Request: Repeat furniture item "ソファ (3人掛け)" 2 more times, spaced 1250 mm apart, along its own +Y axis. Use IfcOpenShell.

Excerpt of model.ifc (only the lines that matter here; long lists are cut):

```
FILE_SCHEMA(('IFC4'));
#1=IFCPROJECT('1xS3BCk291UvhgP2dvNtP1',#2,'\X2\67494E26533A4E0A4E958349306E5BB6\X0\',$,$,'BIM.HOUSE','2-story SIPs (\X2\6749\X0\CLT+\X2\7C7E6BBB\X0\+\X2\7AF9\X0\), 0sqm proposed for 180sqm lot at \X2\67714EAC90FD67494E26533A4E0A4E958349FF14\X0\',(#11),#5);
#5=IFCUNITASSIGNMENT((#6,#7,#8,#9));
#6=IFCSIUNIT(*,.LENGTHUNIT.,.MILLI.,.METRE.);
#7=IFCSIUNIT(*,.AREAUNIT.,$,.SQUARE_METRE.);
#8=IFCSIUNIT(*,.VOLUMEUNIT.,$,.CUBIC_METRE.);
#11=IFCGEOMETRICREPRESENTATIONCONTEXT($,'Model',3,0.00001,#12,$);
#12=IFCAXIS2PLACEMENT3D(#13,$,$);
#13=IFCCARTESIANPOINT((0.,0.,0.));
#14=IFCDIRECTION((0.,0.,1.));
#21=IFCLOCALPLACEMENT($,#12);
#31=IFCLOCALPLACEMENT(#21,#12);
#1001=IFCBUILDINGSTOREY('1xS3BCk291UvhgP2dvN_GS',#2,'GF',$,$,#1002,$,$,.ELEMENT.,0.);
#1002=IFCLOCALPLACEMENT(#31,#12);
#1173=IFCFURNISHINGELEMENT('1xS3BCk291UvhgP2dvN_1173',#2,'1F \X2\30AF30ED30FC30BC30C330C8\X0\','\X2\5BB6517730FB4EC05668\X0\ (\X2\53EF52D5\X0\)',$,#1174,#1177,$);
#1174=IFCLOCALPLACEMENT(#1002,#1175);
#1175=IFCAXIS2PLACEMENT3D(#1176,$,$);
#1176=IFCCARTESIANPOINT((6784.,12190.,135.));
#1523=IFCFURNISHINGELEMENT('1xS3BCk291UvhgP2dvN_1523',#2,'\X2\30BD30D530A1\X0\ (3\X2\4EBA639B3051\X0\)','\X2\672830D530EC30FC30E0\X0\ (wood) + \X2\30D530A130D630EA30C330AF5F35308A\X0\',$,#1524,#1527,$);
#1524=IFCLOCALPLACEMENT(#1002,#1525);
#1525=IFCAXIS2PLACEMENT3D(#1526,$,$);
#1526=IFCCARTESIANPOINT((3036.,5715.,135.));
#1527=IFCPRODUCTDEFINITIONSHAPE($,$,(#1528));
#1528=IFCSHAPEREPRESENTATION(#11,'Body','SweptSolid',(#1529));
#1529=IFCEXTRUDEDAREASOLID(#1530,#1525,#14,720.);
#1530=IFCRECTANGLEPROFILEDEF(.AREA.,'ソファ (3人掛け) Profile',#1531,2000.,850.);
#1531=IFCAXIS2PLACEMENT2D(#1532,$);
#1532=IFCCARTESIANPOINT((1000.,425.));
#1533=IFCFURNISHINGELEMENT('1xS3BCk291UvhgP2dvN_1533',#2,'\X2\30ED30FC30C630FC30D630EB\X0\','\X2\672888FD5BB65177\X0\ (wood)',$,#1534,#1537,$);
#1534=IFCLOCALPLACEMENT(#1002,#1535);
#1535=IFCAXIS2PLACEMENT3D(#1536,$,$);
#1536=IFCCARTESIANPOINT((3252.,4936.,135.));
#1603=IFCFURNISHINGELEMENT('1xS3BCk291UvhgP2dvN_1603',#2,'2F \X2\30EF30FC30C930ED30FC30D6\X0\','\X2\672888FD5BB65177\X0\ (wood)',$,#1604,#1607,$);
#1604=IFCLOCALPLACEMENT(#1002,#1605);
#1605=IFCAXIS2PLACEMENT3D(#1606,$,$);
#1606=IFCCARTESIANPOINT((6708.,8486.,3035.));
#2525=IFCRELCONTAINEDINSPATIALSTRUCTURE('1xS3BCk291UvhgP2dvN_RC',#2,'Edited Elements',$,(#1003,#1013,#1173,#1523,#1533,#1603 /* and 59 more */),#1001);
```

```python
import ifcopenshell
import ifcopenshell.api.geometry
import ifcopenshell.api.root
import ifcopenshell.util.element
import ifcopenshell.util.placement
import ifcopenshell.util.unit

model = ifcopenshell.open("model.ifc")
unit_scale = ifcopenshell.util.unit.calculate_unit_scale(model)


def reuse_history(source, copy):
    """copy_class also copies each property set's owner history, people and application; keep the originals."""
    for rel in copy.IsDefinedBy:
        if rel.is_a("IfcRelDefinesByProperties") and (history := rel.RelatingPropertyDefinition.OwnerHistory):
            rel.RelatingPropertyDefinition.OwnerHistory = source.OwnerHistory
            ifcopenshell.util.element.remove_deep2(model, history)


source = model.by_guid("1xS3BCk291UvhgP2dvN_1523")
base = ifcopenshell.util.placement.get_local_placement(source.ObjectPlacement)
step = base[:3, 1] * 1.25 / unit_scale

for i in range(1, 3):
    copy = ifcopenshell.api.root.copy_class(model, product=source)
    copy.Representation = ifcopenshell.util.element.copy_deep(
        model, source.Representation, exclude=["IfcGeometricRepresentationContext", "IfcRepresentationMap"]
    )
    reuse_history(source, copy)
    matrix = base.copy()
    matrix[:3, 3] += i * step
    print("added at", matrix[:3, 3].round(3) + 0.0)
    ifcopenshell.api.geometry.edit_object_placement(model, product=copy, matrix=matrix, is_si=False)

model.write("model_updated.ifc")
```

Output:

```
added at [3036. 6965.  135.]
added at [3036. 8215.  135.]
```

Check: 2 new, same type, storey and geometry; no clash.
